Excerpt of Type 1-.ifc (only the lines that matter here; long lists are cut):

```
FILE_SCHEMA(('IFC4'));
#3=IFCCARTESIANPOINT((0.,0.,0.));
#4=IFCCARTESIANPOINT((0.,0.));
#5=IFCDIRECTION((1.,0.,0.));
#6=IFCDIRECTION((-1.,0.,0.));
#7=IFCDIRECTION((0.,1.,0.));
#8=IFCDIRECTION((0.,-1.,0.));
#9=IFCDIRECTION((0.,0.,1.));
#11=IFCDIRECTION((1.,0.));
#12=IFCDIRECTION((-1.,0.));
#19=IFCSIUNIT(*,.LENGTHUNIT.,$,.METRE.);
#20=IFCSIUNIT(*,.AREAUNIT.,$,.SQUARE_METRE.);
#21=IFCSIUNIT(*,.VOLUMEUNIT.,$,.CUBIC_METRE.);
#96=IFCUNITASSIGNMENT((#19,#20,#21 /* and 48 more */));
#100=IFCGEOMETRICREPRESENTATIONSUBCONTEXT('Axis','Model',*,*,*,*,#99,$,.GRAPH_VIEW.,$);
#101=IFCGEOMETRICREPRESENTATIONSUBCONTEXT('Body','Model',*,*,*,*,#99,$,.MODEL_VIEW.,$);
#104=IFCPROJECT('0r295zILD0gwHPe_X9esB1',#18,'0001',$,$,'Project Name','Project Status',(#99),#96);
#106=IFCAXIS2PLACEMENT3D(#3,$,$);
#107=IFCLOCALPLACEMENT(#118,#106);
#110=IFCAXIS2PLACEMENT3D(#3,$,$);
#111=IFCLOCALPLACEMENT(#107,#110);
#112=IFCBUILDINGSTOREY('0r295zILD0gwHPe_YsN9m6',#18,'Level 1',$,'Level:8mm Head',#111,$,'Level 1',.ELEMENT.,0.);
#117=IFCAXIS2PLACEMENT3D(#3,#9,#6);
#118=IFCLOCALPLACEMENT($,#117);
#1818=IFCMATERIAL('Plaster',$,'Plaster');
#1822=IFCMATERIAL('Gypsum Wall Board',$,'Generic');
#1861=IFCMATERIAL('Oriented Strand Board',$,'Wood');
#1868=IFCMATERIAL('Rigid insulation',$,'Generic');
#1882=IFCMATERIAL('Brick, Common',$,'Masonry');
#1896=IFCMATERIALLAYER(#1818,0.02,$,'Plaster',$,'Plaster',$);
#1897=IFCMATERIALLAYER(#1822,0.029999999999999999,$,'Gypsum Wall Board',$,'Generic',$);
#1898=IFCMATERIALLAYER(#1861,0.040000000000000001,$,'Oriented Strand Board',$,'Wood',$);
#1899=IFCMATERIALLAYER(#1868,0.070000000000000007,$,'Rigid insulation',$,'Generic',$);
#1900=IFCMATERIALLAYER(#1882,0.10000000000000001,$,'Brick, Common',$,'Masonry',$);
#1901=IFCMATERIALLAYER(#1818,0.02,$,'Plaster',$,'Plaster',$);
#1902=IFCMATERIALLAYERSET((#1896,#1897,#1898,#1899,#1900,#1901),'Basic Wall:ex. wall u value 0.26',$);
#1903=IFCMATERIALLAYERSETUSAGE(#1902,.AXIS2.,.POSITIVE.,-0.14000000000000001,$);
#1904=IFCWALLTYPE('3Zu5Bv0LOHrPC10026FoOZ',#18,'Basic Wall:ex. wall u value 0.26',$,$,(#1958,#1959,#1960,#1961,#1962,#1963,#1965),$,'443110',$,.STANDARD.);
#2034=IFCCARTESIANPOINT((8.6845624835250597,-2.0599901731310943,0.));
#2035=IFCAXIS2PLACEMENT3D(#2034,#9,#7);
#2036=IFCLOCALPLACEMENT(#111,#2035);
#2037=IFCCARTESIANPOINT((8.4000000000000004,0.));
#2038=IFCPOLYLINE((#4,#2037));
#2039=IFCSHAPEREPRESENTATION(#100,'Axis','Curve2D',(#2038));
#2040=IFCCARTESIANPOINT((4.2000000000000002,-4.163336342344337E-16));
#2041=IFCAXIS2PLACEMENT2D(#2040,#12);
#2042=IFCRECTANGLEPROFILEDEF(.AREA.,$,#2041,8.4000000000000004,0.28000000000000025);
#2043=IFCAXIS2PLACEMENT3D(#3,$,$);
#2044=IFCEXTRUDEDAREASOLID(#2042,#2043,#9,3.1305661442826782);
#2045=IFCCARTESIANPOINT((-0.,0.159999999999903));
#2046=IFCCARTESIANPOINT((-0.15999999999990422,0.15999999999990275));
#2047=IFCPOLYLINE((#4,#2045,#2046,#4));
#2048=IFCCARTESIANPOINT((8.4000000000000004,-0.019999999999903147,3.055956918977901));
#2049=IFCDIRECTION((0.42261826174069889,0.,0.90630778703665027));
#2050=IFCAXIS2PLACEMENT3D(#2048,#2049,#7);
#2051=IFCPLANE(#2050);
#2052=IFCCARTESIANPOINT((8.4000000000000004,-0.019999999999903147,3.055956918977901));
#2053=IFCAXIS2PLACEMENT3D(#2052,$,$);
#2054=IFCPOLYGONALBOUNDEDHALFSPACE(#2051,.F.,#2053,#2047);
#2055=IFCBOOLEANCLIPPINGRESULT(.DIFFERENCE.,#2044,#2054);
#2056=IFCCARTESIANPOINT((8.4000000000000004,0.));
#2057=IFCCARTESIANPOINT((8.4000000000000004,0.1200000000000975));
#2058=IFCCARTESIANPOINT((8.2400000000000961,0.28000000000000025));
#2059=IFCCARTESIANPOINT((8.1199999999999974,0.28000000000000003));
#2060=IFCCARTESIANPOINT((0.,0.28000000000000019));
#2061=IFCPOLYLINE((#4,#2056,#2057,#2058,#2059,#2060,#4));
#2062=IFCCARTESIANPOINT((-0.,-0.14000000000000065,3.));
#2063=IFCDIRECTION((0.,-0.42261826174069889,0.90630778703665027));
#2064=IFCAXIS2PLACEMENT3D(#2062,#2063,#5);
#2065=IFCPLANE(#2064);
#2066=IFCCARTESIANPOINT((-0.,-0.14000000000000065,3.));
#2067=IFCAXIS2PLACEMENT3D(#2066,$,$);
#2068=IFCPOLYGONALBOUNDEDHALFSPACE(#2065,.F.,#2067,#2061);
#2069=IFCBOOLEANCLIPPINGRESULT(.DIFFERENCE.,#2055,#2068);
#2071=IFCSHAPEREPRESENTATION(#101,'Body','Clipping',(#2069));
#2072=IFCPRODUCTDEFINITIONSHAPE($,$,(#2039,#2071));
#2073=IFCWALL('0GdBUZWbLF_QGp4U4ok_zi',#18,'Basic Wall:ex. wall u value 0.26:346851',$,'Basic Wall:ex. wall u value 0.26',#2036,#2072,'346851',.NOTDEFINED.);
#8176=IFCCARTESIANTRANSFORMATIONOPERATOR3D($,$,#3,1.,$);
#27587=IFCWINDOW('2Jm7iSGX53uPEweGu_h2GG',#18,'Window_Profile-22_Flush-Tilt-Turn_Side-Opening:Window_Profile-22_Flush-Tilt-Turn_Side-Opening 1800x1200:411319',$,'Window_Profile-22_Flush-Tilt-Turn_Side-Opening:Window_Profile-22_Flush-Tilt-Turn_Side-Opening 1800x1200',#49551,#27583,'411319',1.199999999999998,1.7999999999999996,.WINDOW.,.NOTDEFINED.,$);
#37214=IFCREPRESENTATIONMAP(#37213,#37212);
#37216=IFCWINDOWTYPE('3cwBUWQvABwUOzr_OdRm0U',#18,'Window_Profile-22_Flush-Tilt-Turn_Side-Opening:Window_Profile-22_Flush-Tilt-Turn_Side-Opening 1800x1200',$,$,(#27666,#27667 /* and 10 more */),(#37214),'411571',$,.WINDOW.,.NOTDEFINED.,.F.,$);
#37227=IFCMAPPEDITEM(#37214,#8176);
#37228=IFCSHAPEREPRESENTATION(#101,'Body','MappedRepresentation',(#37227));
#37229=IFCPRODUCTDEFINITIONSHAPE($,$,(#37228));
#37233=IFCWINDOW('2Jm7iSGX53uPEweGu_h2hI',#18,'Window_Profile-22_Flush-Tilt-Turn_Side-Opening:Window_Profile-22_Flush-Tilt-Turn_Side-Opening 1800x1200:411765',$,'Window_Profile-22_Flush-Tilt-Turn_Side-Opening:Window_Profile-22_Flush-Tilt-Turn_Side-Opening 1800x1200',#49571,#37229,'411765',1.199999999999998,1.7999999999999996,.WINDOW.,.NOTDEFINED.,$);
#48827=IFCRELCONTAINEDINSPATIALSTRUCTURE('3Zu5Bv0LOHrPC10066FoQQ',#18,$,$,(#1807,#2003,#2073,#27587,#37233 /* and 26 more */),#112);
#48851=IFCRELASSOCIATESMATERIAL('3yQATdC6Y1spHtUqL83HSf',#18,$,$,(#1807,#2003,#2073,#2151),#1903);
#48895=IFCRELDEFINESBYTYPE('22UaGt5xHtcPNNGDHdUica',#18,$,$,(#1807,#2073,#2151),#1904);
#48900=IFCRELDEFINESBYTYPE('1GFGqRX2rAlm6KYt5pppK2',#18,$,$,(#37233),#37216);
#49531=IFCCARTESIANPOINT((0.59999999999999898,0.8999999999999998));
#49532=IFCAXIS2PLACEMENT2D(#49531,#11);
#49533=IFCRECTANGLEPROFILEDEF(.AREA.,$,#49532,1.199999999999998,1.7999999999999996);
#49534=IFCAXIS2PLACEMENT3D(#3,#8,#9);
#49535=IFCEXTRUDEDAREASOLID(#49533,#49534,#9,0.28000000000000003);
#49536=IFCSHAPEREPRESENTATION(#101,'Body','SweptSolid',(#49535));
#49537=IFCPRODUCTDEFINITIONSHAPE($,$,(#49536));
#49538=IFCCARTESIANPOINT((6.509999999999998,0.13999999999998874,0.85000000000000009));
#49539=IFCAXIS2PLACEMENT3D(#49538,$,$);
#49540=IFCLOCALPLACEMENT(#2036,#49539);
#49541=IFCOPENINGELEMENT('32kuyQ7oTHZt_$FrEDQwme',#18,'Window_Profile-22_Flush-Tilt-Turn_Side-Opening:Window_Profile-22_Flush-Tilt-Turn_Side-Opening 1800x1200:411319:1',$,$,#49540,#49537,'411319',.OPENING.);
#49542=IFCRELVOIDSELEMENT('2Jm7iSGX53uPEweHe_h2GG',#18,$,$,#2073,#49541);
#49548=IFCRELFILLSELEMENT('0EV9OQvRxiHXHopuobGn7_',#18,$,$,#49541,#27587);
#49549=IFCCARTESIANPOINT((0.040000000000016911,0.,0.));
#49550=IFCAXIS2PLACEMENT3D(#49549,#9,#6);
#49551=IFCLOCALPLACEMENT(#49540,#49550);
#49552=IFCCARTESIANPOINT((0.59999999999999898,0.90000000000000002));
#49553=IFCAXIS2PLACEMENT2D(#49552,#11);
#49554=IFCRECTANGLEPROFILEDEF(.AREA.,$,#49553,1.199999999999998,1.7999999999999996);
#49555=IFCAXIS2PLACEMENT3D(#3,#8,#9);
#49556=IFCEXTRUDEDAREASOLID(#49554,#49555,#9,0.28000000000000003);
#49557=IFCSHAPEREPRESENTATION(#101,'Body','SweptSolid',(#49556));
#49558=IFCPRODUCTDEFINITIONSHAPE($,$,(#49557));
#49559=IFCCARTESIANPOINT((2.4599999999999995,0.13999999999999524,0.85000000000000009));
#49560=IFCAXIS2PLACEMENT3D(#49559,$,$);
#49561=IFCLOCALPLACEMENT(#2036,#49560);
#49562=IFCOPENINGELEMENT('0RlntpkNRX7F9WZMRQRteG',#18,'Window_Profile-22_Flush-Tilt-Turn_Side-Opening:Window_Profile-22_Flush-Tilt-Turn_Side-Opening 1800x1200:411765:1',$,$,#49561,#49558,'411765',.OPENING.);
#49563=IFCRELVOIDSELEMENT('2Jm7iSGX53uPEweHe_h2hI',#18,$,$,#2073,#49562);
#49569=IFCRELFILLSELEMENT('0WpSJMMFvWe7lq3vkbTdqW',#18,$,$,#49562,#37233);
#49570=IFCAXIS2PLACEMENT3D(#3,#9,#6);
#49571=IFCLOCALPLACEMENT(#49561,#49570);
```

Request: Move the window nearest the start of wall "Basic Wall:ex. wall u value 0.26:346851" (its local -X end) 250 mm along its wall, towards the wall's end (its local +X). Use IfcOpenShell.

```python
import ifcopenshell
import ifcopenshell.api.geometry
import ifcopenshell.util.placement
import ifcopenshell.util.unit

model = ifcopenshell.open("Type 1-.ifc")
unit_scale = ifcopenshell.util.unit.calculate_unit_scale(model)

window = model.by_guid("2Jm7iSGX53uPEweGu_h2hI")
opening = window.FillsVoids[0].RelatingOpeningElement
wall = opening.VoidsElements[0].RelatingBuildingElement

wall_matrix = ifcopenshell.util.placement.get_local_placement(wall.ObjectPlacement)
shift = wall_matrix[:3, 0] * 0.25 / unit_scale
before = ifcopenshell.util.placement.get_local_placement(window.ObjectPlacement)[:3, 3].copy()

# The window is placed relative to its opening, so it follows when the opening moves.
matrix = ifcopenshell.util.placement.get_local_placement(opening.ObjectPlacement)
matrix[:3, 3] += shift
ifcopenshell.api.geometry.edit_object_placement(
    model, product=opening, matrix=matrix, is_si=False, should_transform_children=True
)

after = ifcopenshell.util.placement.get_local_placement(window.ObjectPlacement)[:3, 3]
print("window moved by", (after - before).round(3) + 0.0)

model.write("Type 1-_updated.ifc")
```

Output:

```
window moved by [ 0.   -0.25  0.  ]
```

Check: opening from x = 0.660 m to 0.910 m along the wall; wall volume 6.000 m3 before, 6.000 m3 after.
